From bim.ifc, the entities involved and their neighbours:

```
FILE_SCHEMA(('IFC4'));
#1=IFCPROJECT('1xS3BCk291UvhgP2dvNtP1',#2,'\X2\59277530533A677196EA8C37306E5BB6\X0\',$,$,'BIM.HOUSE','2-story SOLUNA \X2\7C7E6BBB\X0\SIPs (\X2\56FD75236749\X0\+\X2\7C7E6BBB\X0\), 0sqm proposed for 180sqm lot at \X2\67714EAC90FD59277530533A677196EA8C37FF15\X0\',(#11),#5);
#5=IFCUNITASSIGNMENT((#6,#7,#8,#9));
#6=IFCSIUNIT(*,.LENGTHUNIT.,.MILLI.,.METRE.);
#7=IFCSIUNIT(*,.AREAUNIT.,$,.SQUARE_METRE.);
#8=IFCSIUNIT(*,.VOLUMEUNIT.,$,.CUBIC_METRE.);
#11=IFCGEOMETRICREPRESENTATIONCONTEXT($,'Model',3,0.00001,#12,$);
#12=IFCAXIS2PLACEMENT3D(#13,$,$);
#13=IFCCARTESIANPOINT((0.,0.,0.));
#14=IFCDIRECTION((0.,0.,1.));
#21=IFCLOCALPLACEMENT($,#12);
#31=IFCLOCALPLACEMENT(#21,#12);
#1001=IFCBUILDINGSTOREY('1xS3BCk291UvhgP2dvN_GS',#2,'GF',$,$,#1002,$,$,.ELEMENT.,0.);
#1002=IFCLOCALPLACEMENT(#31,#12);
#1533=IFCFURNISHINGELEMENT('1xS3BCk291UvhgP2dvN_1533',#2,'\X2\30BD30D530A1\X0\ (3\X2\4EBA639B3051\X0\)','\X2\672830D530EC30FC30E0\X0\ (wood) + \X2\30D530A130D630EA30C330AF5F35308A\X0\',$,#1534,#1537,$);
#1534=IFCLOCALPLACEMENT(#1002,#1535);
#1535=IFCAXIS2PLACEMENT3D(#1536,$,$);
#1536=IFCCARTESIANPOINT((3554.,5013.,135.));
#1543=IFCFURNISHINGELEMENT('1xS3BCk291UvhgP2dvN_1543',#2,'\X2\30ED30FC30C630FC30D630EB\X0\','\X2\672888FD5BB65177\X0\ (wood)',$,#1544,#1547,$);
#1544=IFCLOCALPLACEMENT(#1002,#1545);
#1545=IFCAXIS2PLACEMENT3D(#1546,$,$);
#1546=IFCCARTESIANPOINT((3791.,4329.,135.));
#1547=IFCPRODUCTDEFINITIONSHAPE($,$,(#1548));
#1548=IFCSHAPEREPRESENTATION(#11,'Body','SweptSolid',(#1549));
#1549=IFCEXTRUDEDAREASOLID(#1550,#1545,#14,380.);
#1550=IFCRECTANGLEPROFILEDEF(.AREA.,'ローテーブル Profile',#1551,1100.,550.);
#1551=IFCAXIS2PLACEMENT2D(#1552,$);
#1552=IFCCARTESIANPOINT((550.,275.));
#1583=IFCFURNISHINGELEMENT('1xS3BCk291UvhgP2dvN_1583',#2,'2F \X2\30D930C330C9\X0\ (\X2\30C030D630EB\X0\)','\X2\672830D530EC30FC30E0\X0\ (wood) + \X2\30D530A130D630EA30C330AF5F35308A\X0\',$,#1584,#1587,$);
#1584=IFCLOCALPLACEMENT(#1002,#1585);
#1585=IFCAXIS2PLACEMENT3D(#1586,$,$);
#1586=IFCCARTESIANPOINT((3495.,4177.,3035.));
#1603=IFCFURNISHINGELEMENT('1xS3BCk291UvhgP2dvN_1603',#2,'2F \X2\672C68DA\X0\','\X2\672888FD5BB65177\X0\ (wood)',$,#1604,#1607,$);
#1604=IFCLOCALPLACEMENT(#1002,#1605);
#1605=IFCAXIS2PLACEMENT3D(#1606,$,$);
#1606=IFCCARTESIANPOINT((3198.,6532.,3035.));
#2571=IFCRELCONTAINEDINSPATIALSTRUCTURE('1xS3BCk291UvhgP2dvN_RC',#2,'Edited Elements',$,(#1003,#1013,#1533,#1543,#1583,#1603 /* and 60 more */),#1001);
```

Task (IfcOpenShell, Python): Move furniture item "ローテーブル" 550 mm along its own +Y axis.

```python
import ifcopenshell
import ifcopenshell.api.geometry
import ifcopenshell.util.placement

model = ifcopenshell.open("bim.ifc")

item = model.by_guid("1xS3BCk291UvhgP2dvN_1543")
matrix = ifcopenshell.util.placement.get_local_placement(item.ObjectPlacement)
matrix[:3, 3] += matrix[:3, 1] * 550.0
ifcopenshell.api.geometry.edit_object_placement(model, product=item, matrix=matrix, is_si=False)

print(ifcopenshell.util.placement.get_local_placement(item.ObjectPlacement).round(3) + 0.0)

model.write("bim_v2.ifc")
```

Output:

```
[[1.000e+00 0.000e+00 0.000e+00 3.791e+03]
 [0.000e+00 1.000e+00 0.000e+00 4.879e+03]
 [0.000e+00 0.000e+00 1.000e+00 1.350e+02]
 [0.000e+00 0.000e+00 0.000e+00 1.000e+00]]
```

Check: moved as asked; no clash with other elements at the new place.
